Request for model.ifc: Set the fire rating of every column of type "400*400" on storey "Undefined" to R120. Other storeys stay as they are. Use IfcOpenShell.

First a look at what the model holds.

```python
import ifcopenshell
import ifcopenshell.util.element

model = ifcopenshell.open("model.ifc")
print(model.schema)
storey = next(s for s in model.by_type("IfcBuildingStorey") if s.Name == "Undefined")
columns = [e for e in ifcopenshell.util.element.get_decomposition(storey) if e.is_a("IfcColumn")]
seen = {}
for e in columns:
    element_type = ifcopenshell.util.element.get_type(e)
    key = (element_type.Name if element_type != e and element_type else None, ifcopenshell.util.element.get_pset(e, "Pset_ColumnCommon", "FireRating"))
    seen[key] = seen.get(key, 0) + 1
for (name, value), count in sorted(seen.items(), key=str):
    print(count, "x", name, "|", value)
```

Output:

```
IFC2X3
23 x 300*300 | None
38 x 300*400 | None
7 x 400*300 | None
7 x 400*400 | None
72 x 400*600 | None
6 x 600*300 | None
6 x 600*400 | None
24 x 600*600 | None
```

```python
import ifcopenshell
import ifcopenshell.api.pset
import ifcopenshell.util.element

model = ifcopenshell.open("model.ifc")

storey = next(s for s in model.by_type("IfcBuildingStorey") if s.Name == "Undefined")
columns = [e for e in ifcopenshell.util.element.get_decomposition(storey) if e.is_a("IfcColumn")]

count = 0
for e in columns:
    element_type = ifcopenshell.util.element.get_type(e)
    if element_type in (None, e) or element_type.Name != "400*400":
        continue
    # add_pset returns the element's existing set when there is one.
    pset = ifcopenshell.api.pset.add_pset(model, product=e, name="Pset_ColumnCommon")
    ifcopenshell.api.pset.edit_pset(model, pset=pset, properties={"FireRating": "R120"})
    count += 1

print(count, "columns updated")

model.write("model_updated.ifc")
```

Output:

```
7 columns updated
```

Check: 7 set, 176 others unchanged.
